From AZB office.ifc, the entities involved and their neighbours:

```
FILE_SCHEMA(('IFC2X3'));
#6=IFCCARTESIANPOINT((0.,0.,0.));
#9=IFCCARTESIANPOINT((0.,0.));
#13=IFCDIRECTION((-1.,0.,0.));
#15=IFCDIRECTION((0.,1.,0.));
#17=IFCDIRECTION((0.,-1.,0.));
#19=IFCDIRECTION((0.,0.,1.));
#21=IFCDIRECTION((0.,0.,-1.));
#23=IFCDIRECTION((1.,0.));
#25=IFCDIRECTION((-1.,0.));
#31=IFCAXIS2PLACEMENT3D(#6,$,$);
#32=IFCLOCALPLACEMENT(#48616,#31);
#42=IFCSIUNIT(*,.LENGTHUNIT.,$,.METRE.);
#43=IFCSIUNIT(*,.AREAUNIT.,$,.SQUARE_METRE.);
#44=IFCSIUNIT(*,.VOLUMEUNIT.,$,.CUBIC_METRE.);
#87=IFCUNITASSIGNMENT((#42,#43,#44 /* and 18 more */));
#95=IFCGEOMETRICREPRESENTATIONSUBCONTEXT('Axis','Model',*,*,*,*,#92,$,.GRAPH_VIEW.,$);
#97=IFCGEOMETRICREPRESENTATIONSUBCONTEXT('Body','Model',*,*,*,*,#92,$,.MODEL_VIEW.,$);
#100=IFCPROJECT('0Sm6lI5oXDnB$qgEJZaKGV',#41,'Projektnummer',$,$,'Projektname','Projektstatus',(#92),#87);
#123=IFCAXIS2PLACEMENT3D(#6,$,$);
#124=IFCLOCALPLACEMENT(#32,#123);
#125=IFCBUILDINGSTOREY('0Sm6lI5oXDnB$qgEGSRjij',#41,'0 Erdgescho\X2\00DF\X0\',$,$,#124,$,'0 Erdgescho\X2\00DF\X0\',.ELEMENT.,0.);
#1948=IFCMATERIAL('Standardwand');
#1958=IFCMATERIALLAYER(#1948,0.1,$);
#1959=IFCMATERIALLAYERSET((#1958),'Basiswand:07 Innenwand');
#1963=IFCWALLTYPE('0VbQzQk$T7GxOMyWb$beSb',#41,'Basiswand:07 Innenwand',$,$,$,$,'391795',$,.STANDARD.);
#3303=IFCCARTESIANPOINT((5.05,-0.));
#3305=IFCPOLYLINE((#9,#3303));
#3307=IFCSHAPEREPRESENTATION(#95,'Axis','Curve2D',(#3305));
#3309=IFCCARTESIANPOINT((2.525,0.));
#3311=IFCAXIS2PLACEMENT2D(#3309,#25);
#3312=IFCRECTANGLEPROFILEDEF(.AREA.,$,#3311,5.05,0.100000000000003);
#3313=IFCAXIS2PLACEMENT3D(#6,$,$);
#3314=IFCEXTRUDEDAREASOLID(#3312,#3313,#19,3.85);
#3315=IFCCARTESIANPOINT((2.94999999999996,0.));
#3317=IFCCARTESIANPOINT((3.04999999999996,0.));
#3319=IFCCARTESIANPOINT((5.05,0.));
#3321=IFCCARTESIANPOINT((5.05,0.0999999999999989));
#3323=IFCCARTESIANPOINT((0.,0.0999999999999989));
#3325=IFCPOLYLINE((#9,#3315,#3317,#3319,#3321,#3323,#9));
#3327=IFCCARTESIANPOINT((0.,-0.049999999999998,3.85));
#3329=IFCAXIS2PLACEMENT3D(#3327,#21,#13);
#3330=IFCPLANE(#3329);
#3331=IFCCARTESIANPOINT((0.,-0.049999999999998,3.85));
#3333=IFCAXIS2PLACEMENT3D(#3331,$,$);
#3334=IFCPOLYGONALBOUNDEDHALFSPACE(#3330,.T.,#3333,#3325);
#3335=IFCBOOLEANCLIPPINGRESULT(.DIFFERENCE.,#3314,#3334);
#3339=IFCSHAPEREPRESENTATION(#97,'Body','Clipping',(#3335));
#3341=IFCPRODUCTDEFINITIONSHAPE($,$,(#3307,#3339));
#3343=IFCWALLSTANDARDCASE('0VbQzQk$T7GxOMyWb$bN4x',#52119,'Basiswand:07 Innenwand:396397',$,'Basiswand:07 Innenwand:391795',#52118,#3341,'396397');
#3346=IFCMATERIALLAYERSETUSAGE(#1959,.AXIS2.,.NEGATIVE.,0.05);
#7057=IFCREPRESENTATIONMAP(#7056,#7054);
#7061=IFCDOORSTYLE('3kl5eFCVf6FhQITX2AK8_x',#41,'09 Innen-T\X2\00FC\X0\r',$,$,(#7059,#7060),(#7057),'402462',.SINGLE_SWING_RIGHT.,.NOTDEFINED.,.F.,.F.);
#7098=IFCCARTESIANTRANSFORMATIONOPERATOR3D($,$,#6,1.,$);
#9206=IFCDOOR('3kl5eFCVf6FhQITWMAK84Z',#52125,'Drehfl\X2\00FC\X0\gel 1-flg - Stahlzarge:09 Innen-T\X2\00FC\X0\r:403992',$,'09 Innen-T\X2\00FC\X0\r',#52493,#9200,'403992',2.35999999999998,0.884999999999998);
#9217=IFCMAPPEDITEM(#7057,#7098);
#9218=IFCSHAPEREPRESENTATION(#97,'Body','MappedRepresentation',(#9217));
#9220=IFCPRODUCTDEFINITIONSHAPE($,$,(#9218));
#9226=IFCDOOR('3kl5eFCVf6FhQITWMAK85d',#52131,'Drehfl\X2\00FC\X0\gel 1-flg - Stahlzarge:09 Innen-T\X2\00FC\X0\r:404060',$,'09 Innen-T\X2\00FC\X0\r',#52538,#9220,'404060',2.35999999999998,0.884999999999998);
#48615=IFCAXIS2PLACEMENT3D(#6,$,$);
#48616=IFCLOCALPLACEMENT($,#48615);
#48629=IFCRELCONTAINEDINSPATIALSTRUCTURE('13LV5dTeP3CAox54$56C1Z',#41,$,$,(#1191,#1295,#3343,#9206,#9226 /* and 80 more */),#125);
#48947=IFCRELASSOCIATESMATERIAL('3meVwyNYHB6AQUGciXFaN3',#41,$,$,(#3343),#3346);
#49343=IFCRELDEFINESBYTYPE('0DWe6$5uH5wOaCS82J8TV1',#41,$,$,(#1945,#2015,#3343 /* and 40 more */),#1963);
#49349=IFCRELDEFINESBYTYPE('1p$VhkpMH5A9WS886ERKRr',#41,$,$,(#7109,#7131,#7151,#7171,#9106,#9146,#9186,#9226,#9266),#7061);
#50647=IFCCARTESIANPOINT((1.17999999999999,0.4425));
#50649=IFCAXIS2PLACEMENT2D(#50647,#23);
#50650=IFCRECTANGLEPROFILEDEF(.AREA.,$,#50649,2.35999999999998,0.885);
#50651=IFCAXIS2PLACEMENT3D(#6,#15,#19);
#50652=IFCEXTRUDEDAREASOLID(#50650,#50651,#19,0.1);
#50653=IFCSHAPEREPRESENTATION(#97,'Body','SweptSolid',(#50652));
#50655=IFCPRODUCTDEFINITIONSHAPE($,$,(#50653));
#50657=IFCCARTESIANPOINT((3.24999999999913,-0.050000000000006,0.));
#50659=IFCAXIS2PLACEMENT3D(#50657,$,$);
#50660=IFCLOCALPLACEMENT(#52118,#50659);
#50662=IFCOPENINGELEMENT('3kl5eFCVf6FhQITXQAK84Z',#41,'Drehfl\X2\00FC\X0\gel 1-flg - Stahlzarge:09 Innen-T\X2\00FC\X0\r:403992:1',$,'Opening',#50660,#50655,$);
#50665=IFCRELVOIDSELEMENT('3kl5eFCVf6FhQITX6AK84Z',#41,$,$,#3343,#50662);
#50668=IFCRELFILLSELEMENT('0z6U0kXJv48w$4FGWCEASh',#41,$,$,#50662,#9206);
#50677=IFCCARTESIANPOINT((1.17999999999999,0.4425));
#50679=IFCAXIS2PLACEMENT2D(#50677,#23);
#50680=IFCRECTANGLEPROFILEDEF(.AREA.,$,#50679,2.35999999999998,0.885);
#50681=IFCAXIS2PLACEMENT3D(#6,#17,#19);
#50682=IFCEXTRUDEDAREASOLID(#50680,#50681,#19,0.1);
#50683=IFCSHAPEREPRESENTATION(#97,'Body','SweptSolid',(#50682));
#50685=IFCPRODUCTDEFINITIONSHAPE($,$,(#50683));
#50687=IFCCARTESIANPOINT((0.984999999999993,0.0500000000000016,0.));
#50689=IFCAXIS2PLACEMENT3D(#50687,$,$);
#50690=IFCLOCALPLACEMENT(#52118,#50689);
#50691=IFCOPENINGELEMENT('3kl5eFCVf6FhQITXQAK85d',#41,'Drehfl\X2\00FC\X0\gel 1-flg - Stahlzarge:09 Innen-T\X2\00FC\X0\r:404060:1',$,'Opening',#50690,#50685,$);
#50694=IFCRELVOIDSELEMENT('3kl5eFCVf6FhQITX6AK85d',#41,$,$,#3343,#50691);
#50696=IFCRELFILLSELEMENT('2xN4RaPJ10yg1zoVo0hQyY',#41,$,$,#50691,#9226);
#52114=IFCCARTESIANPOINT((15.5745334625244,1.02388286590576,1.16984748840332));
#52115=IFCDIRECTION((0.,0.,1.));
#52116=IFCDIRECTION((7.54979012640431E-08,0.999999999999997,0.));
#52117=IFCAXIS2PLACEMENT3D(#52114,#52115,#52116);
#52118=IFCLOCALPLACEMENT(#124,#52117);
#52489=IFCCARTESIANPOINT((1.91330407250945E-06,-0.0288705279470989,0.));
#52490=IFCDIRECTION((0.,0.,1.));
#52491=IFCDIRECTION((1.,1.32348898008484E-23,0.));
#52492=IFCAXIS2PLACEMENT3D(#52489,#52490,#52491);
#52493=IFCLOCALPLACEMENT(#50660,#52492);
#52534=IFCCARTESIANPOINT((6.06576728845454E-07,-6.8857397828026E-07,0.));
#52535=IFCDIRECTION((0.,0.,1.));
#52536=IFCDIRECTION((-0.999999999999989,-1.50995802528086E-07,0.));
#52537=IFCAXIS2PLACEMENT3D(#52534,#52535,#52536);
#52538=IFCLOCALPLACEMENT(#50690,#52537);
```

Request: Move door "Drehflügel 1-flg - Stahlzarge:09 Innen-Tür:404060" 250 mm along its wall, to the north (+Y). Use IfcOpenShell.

```python
import ifcopenshell
import ifcopenshell.api.geometry
import ifcopenshell.util.placement

model = ifcopenshell.open("AZB office.ifc")

door = model.by_guid("3kl5eFCVf6FhQITWMAK85d")
opening = door.FillsVoids[0].RelatingOpeningElement
wall = opening.VoidsElements[0].RelatingBuildingElement

wall_matrix = ifcopenshell.util.placement.get_local_placement(wall.ObjectPlacement)
shift = wall_matrix[:3, 0] * 0.25
before = ifcopenshell.util.placement.get_local_placement(door.ObjectPlacement)[:3, 3].copy()

# The door is placed relative to its opening, so it follows when the opening moves.
matrix = ifcopenshell.util.placement.get_local_placement(opening.ObjectPlacement)
matrix[:3, 3] += shift
ifcopenshell.api.geometry.edit_object_placement(
    model, product=opening, matrix=matrix, is_si=False, should_transform_children=True
)

after = ifcopenshell.util.placement.get_local_placement(door.ObjectPlacement)[:3, 3]
print("door moved by", (after - before).round(3) + 0.0)

model.write("AZB office_edited.ifc")
```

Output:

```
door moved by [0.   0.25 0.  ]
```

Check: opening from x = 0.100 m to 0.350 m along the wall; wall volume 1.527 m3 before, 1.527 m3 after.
